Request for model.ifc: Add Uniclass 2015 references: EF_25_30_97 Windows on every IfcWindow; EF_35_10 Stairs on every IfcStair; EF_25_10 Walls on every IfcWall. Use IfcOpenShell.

First a look at what the model holds.

```python
import ifcopenshell

model = ifcopenshell.open("model.ifc")
print(model.schema)
print("classifications:", [c.Name for c in model.by_type("IfcClassification")])
for ifc_class in ("IfcDoor", "IfcRoof", "IfcStair", "IfcWall", "IfcWindow"):
    print(ifc_class, len(model.by_type(ifc_class)))
```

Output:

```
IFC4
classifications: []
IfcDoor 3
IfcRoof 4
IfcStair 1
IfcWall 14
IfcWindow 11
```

```python
import ifcopenshell
import ifcopenshell.api.classification

model = ifcopenshell.open("model.ifc")

system = ifcopenshell.api.classification.add_classification(model, classification="Uniclass 2015")

codes = {
    "IfcWindow": ("EF_25_30_97", "Windows"),
    "IfcStair": ("EF_35_10", "Stairs"),
    "IfcWall": ("EF_25_10", "Walls"),
}
for ifc_class, (code, name) in codes.items():
    products = model.by_type(ifc_class)
    ifcopenshell.api.classification.add_reference(
        model, products=products, classification=system, identification=code, name=name
    )
    print(code, len(products))

model.write("model_updated.ifc")
```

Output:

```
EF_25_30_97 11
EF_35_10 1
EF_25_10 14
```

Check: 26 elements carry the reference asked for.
